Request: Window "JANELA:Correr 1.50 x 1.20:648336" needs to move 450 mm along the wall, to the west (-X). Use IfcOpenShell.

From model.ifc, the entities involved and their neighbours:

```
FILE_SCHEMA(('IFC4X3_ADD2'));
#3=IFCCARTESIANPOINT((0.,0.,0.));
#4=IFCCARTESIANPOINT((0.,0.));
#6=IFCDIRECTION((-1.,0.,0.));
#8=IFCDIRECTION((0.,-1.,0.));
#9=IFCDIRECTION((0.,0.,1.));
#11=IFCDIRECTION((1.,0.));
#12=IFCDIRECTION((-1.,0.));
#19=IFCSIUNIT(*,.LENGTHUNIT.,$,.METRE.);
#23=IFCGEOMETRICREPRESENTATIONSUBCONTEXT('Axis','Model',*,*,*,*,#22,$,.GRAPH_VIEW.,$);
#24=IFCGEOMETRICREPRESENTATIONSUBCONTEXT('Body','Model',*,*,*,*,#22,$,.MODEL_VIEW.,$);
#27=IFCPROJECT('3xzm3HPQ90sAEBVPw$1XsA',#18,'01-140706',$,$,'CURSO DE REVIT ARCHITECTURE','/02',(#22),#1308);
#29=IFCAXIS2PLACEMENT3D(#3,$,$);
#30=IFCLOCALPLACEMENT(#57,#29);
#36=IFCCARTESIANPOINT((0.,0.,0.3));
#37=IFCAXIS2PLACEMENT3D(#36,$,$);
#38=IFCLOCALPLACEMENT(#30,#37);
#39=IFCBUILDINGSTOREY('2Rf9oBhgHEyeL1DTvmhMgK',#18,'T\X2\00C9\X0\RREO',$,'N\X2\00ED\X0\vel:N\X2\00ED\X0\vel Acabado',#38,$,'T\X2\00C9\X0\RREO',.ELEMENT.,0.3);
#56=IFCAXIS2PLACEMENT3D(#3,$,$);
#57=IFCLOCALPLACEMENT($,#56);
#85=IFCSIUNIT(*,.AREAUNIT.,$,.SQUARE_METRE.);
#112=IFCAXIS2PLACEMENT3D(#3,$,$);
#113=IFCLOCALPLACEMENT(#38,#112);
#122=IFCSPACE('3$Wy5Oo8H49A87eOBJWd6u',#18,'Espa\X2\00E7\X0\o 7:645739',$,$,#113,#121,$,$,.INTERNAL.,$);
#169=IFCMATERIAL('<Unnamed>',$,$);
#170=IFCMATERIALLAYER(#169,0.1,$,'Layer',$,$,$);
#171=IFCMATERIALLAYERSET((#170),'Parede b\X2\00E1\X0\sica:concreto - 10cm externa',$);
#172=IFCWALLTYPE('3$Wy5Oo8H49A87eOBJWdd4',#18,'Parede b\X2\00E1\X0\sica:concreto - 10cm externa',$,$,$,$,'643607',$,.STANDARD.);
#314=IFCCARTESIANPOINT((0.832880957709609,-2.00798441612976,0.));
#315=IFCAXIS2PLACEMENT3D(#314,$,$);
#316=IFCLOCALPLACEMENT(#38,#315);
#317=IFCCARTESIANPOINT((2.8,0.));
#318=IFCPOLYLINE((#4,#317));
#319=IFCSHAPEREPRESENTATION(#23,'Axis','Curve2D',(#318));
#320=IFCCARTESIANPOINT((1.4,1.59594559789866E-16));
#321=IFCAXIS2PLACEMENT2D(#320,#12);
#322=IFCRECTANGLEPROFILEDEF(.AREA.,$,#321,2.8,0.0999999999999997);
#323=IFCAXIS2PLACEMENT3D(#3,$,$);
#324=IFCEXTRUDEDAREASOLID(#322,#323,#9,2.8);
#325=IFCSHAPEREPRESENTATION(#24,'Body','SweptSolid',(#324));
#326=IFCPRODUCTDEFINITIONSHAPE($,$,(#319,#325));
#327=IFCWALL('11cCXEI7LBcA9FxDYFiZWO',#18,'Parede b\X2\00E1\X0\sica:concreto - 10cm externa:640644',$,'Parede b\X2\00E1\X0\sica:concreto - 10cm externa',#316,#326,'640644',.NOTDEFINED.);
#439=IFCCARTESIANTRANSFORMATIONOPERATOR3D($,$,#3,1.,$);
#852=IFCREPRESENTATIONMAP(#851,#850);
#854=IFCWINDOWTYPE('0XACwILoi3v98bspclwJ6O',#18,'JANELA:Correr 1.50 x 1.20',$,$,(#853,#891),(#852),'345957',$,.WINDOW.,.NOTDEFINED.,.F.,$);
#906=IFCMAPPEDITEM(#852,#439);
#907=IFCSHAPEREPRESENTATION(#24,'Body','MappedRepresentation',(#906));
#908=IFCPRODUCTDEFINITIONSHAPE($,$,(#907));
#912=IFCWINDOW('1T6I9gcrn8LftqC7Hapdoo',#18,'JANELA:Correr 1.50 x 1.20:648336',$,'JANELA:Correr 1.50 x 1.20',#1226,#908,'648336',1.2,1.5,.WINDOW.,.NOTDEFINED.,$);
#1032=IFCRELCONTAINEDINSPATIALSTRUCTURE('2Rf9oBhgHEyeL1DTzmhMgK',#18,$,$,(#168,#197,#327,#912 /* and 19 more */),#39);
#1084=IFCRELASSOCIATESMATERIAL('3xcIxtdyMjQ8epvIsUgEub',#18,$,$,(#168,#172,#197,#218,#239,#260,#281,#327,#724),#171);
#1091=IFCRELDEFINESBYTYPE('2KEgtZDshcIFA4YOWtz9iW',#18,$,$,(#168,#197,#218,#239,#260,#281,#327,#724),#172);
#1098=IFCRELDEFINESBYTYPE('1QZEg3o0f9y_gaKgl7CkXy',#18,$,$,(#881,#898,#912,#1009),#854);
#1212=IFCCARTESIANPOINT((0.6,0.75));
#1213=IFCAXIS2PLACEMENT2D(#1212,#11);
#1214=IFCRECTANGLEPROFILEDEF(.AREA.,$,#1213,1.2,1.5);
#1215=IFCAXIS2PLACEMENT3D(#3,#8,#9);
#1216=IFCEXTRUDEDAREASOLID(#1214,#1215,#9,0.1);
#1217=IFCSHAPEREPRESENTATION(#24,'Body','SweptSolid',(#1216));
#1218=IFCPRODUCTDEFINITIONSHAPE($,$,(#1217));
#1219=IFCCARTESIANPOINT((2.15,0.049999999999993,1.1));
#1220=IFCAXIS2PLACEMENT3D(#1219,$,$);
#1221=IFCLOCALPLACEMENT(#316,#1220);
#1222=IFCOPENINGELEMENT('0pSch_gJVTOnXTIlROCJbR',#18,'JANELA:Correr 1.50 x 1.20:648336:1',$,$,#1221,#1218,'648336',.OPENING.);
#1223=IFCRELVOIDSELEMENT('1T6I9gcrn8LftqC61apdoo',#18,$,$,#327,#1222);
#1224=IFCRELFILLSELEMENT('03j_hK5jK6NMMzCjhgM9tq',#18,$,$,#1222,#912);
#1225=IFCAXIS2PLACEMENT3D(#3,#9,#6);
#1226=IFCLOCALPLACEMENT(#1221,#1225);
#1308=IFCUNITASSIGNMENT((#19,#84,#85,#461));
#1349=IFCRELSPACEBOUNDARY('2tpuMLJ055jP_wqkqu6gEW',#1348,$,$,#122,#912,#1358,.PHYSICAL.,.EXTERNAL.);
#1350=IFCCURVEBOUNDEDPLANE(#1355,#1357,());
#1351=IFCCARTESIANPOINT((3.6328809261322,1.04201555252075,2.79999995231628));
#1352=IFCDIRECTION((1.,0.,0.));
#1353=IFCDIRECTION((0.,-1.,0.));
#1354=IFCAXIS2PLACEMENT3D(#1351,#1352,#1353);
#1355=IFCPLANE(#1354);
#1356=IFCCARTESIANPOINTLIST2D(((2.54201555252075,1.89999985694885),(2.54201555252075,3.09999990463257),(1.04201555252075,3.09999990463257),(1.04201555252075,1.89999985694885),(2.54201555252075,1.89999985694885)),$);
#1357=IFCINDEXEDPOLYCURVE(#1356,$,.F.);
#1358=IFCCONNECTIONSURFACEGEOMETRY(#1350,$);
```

```python
import numpy as np
import ifcopenshell
import ifcopenshell.api.geometry
import ifcopenshell.util.placement
import ifcopenshell.util.unit

model = ifcopenshell.open("model.ifc")
unit_scale = ifcopenshell.util.unit.calculate_unit_scale(model)

window = model.by_id(912)
opening = window.FillsVoids[0].RelatingOpeningElement
wall = opening.VoidsElements[0].RelatingBuildingElement

wall_matrix = ifcopenshell.util.placement.get_local_placement(wall.ObjectPlacement)
shift = wall_matrix[:3, 0] * -0.45 / unit_scale
before = ifcopenshell.util.placement.get_local_placement(window.ObjectPlacement)[:3, 3].copy()

# The window is placed relative to its opening, so it follows when the opening moves.
matrix = ifcopenshell.util.placement.get_local_placement(opening.ObjectPlacement)
matrix[:3, 3] += shift
ifcopenshell.api.geometry.edit_object_placement(
    model, product=opening, matrix=matrix, is_si=False, should_transform_children=True
)

# Space boundary surfaces are stored in each space's coordinates; move them too.
for rel in window.ProvidesBoundaries:
    if not rel.ConnectionGeometry:
        continue
    surface = rel.ConnectionGeometry.SurfaceOnRelatingElement.BasisSurface
    space_matrix = ifcopenshell.util.placement.get_local_placement(rel.RelatingSpace.ObjectPlacement)
    point = np.array(surface.Position.Location.Coordinates) + space_matrix[:3, :3].T @ shift
    surface.Position = model.createIfcAxis2Placement3D(
        model.createIfcCartesianPoint(point.tolist()), surface.Position.Axis, surface.Position.RefDirection
    )

after = ifcopenshell.util.placement.get_local_placement(window.ObjectPlacement)[:3, 3]
print("window moved by", (after - before).round(3) + 0.0)

model.write("model_rev.ifc")
```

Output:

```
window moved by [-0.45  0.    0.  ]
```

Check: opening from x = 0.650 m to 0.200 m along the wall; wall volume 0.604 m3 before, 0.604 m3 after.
